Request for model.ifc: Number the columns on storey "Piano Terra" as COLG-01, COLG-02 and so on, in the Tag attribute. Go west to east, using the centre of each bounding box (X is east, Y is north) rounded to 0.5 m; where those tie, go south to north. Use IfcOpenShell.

First a look at what the model holds.

```python
import ifcopenshell
import ifcopenshell.util.element
import ifcopenshell.util.placement

model = ifcopenshell.open("model.ifc")
print(model.schema)
storey = next(s for s in model.by_type("IfcBuildingStorey") if s.Name == "Piano Terra")
columns = [e for e in ifcopenshell.util.element.get_decomposition(storey) if e.is_a("IfcColumn")]
for e in sorted(columns, key=lambda e: e.id()):
    origin = ifcopenshell.util.placement.get_local_placement(e.ObjectPlacement)[:3, 3]
    print(e.id(), e.Tag, e.Name, origin.round(2) + 0.0, sep=" | ")
```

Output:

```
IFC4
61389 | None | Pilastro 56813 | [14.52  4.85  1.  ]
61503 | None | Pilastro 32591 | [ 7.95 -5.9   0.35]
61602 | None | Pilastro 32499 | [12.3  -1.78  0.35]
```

```python
import ifcopenshell
import ifcopenshell.geom
import ifcopenshell.util.element
import ifcopenshell.util.shape

model = ifcopenshell.open("model.ifc")
settings = ifcopenshell.geom.settings()
settings.set("use-world-coords", True)


def centre(element):
    shape = ifcopenshell.geom.create_shape(settings, element)
    return ifcopenshell.util.shape.get_bbox_centroid(shape.geometry)


storey = next(s for s in model.by_type("IfcBuildingStorey") if s.Name == "Piano Terra")
columns = [e for e in ifcopenshell.util.element.get_decomposition(storey) if e.is_a("IfcColumn")]

# Insertion points can sit at a corner or the storey origin, so sort by the geometry (in metres).
centres = {e: centre(e) for e in columns}
columns.sort(key=lambda e: (round(centres[e][0] / 0.5), centres[e][1]))

for i, e in enumerate(columns, start=1):
    number = f"COLG-{i:02d}"
    e.Tag = number
    print(e.id(), number)

model.write("model_updated.ifc")
```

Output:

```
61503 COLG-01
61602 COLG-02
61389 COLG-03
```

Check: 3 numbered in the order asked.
